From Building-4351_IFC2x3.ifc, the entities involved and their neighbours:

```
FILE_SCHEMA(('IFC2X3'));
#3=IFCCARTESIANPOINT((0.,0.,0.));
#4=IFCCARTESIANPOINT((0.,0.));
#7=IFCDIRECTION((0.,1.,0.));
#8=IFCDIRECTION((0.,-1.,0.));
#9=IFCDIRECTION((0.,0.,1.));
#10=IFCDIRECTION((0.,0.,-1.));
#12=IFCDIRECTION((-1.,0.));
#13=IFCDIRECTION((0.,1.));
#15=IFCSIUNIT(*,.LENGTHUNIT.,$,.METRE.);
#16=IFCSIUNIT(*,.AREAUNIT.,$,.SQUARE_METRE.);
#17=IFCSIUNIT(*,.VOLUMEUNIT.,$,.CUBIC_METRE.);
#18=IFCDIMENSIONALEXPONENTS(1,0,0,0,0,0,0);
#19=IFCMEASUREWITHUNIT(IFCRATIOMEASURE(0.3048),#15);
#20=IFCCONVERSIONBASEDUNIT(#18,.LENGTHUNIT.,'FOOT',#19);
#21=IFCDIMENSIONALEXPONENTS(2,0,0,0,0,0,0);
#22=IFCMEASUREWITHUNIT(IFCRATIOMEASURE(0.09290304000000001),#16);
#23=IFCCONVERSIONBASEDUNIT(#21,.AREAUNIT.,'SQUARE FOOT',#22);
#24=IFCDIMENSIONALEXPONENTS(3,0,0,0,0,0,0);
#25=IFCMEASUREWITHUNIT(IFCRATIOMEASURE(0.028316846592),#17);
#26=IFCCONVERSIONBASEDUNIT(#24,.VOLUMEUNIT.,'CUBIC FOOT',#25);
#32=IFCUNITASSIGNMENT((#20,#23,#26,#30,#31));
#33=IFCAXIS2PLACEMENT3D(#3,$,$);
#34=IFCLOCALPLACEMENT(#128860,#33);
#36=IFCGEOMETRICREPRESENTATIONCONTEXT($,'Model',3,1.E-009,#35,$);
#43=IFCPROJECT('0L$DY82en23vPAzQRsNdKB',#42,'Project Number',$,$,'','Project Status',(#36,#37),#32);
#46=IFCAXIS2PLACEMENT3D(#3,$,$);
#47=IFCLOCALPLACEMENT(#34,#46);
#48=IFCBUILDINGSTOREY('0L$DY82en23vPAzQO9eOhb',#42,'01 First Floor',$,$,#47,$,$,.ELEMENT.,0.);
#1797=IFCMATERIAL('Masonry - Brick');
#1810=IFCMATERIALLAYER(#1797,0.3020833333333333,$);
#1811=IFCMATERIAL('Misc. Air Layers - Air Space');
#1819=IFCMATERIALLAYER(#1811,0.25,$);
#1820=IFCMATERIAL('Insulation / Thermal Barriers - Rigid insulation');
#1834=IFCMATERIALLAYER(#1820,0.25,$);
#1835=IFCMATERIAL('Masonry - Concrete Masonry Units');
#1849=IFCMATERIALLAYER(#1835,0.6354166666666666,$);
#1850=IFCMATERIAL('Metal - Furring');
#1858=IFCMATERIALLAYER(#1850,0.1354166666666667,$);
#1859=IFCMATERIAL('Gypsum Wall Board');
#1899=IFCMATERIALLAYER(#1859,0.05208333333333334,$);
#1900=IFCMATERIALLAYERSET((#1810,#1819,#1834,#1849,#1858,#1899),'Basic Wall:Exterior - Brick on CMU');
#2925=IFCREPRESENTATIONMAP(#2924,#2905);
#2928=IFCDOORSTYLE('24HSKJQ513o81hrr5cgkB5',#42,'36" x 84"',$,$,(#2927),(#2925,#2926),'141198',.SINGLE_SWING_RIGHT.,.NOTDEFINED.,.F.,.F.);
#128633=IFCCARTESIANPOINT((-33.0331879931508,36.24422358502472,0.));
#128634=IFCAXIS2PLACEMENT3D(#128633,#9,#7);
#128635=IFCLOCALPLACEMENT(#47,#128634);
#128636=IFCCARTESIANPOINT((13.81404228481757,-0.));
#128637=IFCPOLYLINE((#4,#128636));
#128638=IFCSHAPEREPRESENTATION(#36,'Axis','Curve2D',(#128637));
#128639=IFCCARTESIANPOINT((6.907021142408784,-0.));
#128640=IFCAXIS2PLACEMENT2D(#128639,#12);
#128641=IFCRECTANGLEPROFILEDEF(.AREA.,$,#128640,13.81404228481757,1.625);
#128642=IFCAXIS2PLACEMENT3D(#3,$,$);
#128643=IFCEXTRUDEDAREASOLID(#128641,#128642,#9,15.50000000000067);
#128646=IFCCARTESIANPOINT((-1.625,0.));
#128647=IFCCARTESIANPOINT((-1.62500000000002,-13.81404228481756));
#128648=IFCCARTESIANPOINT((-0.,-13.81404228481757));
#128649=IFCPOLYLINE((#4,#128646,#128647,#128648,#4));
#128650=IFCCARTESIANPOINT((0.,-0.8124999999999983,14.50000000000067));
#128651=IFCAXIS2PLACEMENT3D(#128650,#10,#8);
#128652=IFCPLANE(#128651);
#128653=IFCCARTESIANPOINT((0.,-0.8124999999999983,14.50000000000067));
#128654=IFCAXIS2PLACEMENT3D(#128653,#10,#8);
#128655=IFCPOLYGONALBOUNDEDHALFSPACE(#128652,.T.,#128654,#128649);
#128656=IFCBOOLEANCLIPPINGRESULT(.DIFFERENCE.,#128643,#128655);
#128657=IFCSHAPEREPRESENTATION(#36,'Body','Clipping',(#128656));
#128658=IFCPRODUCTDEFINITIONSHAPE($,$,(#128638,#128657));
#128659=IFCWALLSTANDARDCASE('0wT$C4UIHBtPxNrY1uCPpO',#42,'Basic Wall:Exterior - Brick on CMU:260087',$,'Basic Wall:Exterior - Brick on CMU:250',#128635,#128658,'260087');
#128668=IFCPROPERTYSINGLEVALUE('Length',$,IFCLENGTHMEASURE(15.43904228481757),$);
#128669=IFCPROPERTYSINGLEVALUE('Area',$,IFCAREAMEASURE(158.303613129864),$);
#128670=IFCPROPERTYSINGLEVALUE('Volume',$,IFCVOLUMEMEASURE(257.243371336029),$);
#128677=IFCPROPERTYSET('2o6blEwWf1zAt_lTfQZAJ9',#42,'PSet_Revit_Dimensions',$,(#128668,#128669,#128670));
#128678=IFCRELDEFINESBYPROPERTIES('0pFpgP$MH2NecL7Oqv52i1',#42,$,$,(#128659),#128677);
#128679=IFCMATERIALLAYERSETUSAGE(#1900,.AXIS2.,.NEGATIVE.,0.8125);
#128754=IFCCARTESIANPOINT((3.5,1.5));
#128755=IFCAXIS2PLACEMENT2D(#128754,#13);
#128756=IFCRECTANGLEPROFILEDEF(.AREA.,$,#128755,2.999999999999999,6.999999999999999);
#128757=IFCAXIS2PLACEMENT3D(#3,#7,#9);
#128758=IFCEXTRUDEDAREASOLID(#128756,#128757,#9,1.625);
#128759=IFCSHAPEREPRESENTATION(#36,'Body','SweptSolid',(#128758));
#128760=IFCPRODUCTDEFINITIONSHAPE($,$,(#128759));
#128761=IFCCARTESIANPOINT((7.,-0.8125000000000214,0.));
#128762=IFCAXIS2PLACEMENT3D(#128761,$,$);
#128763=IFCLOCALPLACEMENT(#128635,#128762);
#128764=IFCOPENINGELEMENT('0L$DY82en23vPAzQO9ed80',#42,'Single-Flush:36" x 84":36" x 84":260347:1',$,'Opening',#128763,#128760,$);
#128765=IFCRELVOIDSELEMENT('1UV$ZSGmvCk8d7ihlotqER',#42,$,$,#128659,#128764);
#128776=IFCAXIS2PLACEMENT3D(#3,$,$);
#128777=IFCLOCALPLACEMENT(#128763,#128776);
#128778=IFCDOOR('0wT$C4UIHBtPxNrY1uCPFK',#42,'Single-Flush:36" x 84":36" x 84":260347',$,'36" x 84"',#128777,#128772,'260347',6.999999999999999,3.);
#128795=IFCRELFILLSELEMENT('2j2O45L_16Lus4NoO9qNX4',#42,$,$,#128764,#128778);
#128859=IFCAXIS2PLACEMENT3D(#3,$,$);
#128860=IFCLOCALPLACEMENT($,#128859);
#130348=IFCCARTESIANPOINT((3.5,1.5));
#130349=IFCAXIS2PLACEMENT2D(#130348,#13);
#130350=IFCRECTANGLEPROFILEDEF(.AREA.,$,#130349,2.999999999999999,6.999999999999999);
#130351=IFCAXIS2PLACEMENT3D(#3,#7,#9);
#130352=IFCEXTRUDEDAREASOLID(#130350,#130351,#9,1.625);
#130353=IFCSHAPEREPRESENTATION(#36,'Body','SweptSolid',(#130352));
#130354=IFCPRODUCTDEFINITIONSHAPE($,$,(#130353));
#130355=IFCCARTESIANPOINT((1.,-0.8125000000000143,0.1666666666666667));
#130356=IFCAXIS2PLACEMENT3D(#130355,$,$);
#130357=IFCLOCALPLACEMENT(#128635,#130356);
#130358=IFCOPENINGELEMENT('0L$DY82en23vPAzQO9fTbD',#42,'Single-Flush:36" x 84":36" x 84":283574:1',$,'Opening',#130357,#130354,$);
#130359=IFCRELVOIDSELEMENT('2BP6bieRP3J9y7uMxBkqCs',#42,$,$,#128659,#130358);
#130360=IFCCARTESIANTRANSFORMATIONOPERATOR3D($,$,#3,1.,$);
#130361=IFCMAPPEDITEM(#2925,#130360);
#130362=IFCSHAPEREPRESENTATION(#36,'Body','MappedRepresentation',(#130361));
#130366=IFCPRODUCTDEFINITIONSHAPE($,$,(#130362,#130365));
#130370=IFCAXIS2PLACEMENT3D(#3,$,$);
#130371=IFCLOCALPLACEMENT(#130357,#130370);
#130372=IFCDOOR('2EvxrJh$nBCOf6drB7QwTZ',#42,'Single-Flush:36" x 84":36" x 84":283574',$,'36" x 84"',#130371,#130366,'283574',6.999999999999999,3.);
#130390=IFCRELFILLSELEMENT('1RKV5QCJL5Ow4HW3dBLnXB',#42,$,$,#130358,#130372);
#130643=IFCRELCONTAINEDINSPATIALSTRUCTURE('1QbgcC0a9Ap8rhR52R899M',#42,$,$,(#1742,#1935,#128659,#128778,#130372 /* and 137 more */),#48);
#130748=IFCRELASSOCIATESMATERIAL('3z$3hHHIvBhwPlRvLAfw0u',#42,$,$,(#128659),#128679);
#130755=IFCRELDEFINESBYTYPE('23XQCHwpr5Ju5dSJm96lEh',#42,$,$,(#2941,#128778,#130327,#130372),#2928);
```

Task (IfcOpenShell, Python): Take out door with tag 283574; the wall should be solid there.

```python
import ifcopenshell
import ifcopenshell.api.feature
import ifcopenshell.api.pset
import ifcopenshell.api.root
import ifcopenshell.geom
import ifcopenshell.util.element
import ifcopenshell.util.shape
import ifcopenshell.util.unit

model = ifcopenshell.open("Building-4351_IFC2x3.ifc")
area_scale = ifcopenshell.util.unit.calculate_unit_scale(model, "AREAUNIT")
volume_scale = ifcopenshell.util.unit.calculate_unit_scale(model, "VOLUMEUNIT")
settings = ifcopenshell.geom.settings()


def volume(element):
    """Net volume in cubic metres, openings subtracted."""
    shape = ifcopenshell.geom.create_shape(settings, element)
    return ifcopenshell.util.shape.get_volume(shape.geometry)


door = model.by_guid("2EvxrJh$nBCOf6drB7QwTZ")
opening = door.FillsVoids[0].RelatingOpeningElement
wall = opening.VoidsElements[0].RelatingBuildingElement
before = volume(wall)

ifcopenshell.api.root.remove_product(model, product=door)
ifcopenshell.api.feature.remove_feature(model, feature=opening)

after = volume(wall)
thickness = 0.4953  # wall thickness in metres

# Update the wall's stored quantities.
pset = model.by_id(ifcopenshell.util.element.get_pset(wall, "PSet_Revit_Dimensions", should_inherit=False)["id"])
ifcopenshell.api.pset.edit_pset(model, pset=pset, properties={
    "Area": model.create_entity("IfcAreaMeasure", after / thickness / area_scale),
    "Volume": model.create_entity("IfcVolumeMeasure", after / volume_scale),
})

print(f"wall volume {before:.3f} -> {after:.3f} m3")

model.write("Building-4351_IFC2x3_updated.ifc")
```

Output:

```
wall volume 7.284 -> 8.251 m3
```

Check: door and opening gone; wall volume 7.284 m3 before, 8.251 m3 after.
